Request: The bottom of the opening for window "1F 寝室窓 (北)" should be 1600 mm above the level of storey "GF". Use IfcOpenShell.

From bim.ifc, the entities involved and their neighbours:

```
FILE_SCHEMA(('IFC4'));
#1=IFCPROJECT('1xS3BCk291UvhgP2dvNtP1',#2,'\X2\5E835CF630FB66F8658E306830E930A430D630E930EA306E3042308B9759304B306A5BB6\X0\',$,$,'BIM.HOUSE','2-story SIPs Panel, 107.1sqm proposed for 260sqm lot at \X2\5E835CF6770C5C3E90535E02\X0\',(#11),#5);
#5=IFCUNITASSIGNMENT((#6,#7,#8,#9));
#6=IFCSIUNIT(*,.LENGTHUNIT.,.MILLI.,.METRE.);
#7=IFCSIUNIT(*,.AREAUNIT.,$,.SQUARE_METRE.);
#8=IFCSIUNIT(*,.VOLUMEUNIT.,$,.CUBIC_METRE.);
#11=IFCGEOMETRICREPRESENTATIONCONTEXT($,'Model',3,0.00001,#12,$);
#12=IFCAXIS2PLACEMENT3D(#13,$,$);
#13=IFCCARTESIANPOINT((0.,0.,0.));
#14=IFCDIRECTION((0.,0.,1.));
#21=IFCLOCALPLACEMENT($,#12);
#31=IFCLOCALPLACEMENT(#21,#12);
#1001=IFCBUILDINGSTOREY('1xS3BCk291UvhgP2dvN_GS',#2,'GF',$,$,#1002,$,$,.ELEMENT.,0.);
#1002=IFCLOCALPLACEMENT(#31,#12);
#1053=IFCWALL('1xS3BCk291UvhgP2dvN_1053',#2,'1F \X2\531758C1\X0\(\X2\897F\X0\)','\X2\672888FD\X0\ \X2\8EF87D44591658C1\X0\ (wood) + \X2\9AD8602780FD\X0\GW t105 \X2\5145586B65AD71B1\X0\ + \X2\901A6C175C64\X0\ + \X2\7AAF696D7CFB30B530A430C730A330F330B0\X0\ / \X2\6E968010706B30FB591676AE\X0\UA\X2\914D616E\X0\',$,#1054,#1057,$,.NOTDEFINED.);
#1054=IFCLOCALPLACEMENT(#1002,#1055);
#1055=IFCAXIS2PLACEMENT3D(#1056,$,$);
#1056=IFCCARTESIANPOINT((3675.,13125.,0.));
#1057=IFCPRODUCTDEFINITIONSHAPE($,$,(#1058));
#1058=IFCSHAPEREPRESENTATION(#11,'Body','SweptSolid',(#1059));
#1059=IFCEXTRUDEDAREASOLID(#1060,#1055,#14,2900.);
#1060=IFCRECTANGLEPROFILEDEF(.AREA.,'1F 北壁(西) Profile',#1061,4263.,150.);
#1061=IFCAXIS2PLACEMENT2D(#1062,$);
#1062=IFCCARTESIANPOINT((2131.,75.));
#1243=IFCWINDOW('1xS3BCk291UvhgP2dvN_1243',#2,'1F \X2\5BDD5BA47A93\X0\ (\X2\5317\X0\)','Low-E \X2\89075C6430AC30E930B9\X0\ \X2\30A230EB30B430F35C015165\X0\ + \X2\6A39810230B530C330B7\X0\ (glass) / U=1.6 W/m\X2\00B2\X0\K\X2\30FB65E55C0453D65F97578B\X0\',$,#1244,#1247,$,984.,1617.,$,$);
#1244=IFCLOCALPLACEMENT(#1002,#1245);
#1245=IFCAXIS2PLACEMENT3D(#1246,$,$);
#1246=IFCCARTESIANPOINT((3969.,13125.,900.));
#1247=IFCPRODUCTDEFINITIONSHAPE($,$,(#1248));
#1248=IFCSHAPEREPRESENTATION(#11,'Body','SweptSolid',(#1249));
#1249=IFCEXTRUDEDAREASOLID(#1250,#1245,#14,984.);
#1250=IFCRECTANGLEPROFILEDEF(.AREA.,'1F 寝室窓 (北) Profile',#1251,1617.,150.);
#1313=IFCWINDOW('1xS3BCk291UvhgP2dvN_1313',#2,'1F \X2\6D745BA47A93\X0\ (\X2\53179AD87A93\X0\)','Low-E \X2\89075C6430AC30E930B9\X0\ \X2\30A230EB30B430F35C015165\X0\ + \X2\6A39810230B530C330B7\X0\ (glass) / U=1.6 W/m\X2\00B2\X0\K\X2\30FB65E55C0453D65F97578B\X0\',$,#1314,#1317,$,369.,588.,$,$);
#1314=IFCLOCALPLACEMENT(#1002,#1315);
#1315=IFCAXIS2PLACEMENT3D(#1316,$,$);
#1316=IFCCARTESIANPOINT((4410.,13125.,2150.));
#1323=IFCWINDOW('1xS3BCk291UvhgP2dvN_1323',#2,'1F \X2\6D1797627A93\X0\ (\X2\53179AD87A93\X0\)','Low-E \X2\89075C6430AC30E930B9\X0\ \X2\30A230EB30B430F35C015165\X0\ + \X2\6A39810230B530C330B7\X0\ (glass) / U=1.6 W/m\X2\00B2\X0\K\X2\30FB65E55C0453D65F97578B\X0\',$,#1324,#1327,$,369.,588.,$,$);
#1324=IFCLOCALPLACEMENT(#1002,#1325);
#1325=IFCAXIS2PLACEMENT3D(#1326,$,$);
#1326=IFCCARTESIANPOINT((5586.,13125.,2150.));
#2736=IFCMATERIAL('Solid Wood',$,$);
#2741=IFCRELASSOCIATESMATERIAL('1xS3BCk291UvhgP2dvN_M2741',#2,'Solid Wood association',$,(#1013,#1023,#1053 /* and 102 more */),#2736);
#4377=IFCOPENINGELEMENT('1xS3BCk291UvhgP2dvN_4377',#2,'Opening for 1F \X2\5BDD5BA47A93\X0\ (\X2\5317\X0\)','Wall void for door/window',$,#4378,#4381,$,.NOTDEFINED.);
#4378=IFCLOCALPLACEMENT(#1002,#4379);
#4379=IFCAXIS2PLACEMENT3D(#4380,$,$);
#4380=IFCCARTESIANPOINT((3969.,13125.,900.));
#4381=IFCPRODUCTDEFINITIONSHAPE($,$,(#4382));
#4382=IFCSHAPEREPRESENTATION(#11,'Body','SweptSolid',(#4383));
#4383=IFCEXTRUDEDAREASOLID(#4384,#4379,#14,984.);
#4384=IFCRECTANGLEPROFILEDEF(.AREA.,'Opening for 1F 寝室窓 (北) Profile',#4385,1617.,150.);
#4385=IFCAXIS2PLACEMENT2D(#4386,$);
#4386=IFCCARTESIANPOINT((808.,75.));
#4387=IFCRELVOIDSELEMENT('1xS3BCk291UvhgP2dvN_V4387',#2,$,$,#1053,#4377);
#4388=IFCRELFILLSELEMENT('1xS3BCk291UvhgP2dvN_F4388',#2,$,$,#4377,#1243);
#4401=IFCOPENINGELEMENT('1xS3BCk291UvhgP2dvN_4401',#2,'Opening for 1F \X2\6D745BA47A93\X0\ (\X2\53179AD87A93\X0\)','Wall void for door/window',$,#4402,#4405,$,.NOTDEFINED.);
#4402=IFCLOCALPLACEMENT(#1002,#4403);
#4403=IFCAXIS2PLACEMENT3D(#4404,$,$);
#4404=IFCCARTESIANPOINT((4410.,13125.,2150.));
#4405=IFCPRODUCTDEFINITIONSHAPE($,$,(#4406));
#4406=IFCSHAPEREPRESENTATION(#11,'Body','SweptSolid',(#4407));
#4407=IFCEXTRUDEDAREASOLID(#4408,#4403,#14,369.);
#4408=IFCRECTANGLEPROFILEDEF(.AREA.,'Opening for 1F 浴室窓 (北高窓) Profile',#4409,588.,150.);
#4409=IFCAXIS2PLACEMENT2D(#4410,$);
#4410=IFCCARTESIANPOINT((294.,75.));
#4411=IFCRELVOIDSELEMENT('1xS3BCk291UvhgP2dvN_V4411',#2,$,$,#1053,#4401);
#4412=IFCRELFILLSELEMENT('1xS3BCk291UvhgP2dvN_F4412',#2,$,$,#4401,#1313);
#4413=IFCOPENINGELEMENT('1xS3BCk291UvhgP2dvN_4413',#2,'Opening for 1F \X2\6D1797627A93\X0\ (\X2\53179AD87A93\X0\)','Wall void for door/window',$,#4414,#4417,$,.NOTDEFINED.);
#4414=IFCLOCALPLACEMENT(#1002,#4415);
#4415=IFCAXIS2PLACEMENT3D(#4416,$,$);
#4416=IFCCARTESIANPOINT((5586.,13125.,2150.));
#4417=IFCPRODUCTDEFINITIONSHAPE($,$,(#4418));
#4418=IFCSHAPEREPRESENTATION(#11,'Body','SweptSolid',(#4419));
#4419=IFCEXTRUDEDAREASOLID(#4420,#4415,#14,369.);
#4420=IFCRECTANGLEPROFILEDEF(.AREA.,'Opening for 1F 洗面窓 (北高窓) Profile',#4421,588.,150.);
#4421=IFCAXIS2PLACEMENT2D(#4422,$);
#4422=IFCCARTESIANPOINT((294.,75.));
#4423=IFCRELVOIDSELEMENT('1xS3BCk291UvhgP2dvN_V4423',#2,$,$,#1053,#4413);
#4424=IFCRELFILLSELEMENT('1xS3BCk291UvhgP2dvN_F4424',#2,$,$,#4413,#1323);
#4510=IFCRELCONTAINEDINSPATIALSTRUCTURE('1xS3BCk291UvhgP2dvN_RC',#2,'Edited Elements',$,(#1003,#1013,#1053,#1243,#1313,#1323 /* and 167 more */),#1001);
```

```python
import numpy as np
import ifcopenshell
import ifcopenshell.api.geometry
import ifcopenshell.geom
import ifcopenshell.util.element
import ifcopenshell.util.placement
import ifcopenshell.util.shape
import ifcopenshell.util.unit

model = ifcopenshell.open("bim.ifc")
unit_scale = ifcopenshell.util.unit.calculate_unit_scale(model)

window = model.by_guid("1xS3BCk291UvhgP2dvN_1243")
opening = window.FillsVoids[0].RelatingOpeningElement
storey = ifcopenshell.util.element.get_container(window, ifc_class="IfcBuildingStorey")
level = ifcopenshell.util.placement.get_local_placement(storey.ObjectPlacement)[2, 3]

# The opening's origin need not be at the sill, so measure its lowest point.
shape = ifcopenshell.geom.create_shape(ifcopenshell.geom.settings(), opening)
bottom = ifcopenshell.util.shape.get_shape_bottom_elevation(shape, shape.geometry) / unit_scale
dz = level + 1.6 / unit_scale - bottom

shift = np.array([0.0, 0.0, dz])
# The window is not placed relative to its opening, so move both.
for product in (opening, window):
    matrix = ifcopenshell.util.placement.get_local_placement(product.ObjectPlacement)
    matrix[:3, 3] += shift
    ifcopenshell.api.geometry.edit_object_placement(model, product=product, matrix=matrix, is_si=False)

print(f"moved by {dz * unit_scale:+.3f} m")

model.write("bim_updated.ifc")
```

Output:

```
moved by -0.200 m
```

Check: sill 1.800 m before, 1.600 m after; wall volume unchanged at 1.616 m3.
